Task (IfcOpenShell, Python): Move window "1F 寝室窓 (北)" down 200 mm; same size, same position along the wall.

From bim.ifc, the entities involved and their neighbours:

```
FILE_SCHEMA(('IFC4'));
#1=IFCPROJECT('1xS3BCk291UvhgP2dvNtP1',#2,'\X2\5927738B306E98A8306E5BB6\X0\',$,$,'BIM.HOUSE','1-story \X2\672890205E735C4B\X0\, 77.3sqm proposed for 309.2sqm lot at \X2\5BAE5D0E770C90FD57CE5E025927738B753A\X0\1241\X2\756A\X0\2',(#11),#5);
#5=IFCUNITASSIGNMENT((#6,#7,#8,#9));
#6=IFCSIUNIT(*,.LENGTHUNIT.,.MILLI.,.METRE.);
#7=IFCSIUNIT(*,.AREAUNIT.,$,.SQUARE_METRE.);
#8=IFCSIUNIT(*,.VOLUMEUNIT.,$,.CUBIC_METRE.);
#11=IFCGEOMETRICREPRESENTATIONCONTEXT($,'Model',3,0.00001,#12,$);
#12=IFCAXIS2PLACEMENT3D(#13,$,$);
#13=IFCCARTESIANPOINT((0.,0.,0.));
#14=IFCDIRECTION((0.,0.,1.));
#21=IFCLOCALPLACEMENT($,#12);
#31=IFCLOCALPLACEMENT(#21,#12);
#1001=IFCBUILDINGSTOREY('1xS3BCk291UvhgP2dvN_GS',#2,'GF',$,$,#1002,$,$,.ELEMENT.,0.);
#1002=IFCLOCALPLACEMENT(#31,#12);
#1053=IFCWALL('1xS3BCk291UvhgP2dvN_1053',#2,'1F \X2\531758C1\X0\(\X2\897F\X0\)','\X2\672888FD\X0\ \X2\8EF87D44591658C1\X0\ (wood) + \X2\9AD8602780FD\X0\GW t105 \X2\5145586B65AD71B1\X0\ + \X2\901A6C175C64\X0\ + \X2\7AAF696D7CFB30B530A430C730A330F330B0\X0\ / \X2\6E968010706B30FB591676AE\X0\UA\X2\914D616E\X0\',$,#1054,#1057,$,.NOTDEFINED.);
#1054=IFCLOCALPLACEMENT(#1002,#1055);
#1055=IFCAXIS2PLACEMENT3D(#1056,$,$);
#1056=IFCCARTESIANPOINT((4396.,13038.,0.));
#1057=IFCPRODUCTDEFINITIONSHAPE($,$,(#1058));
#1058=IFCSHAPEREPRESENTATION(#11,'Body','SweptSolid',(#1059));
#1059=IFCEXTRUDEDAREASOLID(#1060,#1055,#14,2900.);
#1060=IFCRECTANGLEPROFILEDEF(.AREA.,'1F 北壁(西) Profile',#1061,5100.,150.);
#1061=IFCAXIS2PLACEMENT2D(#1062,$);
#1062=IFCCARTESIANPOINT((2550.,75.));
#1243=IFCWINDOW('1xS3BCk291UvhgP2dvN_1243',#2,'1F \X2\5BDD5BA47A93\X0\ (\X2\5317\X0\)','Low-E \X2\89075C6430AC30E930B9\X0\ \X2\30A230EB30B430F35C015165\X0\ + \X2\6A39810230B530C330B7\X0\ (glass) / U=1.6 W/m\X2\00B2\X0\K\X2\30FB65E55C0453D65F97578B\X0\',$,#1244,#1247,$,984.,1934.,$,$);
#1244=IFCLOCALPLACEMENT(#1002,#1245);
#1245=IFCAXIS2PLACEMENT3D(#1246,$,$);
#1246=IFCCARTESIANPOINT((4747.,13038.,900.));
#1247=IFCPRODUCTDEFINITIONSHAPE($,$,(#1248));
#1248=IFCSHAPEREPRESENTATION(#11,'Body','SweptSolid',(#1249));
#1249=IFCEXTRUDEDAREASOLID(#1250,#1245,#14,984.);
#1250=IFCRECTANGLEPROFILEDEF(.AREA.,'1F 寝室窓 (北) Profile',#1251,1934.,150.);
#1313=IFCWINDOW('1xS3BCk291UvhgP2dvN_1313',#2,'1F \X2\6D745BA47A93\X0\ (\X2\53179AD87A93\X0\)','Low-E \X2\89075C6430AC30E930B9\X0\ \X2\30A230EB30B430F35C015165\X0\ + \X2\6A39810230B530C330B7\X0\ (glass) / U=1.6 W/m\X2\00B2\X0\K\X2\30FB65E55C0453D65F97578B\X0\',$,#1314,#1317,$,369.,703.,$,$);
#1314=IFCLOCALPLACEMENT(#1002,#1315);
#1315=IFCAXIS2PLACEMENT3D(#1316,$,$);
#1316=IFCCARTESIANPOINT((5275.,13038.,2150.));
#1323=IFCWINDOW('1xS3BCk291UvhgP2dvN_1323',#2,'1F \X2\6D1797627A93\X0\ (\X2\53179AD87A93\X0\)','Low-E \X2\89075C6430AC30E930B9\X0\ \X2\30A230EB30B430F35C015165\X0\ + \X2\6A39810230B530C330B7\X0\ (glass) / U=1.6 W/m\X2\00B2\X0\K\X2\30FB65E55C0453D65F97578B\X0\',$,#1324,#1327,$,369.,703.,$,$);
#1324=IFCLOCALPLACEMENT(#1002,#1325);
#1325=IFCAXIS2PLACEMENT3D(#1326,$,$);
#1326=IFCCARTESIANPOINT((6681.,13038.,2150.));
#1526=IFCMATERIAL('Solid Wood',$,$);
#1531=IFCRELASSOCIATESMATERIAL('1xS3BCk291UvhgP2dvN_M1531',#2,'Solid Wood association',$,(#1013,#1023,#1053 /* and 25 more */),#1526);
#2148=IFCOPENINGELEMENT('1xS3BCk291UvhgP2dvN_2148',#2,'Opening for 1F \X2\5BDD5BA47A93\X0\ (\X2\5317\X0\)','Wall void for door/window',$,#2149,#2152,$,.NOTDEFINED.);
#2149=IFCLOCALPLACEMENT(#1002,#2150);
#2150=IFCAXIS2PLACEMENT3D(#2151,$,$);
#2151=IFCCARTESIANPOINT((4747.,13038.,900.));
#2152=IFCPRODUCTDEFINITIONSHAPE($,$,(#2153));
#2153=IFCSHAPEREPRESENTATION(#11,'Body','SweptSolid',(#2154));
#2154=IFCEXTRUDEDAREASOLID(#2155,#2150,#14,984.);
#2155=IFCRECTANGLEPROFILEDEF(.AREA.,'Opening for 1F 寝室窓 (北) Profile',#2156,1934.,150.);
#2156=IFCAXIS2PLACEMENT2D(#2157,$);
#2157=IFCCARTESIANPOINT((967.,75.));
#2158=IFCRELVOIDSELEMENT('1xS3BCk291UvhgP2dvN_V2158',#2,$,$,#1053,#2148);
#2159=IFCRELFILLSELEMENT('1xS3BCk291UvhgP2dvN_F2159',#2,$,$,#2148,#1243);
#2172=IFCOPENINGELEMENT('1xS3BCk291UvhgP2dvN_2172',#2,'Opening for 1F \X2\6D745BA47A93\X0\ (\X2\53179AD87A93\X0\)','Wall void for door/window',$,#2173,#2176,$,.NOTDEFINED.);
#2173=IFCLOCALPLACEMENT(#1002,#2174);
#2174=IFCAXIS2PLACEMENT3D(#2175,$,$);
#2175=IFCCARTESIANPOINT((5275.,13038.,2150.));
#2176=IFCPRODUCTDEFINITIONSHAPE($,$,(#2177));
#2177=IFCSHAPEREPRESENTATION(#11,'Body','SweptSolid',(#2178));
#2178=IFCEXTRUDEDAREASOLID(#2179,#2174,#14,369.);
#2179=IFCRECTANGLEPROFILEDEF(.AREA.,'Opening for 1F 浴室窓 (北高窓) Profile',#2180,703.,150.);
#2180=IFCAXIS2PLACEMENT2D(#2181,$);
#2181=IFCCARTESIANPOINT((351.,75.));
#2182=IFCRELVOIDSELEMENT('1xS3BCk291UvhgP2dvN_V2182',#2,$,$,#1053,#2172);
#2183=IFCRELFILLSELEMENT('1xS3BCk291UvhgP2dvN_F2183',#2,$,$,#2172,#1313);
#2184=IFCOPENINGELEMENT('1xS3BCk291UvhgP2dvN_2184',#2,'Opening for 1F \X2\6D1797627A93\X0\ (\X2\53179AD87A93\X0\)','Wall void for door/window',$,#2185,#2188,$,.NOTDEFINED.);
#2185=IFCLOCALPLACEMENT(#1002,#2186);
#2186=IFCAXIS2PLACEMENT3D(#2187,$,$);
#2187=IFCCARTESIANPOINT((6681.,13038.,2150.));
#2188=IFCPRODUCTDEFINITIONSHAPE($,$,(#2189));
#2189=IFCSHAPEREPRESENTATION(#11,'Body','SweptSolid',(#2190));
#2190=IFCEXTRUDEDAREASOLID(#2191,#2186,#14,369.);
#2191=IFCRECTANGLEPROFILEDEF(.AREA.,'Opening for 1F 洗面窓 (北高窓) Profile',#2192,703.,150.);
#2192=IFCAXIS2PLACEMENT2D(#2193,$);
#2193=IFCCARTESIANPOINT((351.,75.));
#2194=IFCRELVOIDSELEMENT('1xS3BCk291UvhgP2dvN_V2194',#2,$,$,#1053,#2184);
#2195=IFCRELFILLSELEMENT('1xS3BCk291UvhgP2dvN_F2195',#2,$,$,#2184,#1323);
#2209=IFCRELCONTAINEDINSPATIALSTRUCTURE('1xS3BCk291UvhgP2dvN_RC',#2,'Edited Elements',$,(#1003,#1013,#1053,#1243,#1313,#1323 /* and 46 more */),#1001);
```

```python
import numpy as np
import ifcopenshell
import ifcopenshell.api.geometry
import ifcopenshell.util.placement
import ifcopenshell.util.unit

model = ifcopenshell.open("bim.ifc")
unit_scale = ifcopenshell.util.unit.calculate_unit_scale(model)

window = model.by_guid("1xS3BCk291UvhgP2dvN_1243")
opening = window.FillsVoids[0].RelatingOpeningElement
dz = -200.0

shift = np.array([0.0, 0.0, dz])
# The window is not placed relative to its opening, so move both.
for product in (opening, window):
    matrix = ifcopenshell.util.placement.get_local_placement(product.ObjectPlacement)
    matrix[:3, 3] += shift
    ifcopenshell.api.geometry.edit_object_placement(model, product=product, matrix=matrix, is_si=False)

print(f"moved by {dz * unit_scale:+.3f} m")

model.write("bim_edited.ifc")
```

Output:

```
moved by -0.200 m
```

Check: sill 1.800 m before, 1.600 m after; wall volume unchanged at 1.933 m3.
